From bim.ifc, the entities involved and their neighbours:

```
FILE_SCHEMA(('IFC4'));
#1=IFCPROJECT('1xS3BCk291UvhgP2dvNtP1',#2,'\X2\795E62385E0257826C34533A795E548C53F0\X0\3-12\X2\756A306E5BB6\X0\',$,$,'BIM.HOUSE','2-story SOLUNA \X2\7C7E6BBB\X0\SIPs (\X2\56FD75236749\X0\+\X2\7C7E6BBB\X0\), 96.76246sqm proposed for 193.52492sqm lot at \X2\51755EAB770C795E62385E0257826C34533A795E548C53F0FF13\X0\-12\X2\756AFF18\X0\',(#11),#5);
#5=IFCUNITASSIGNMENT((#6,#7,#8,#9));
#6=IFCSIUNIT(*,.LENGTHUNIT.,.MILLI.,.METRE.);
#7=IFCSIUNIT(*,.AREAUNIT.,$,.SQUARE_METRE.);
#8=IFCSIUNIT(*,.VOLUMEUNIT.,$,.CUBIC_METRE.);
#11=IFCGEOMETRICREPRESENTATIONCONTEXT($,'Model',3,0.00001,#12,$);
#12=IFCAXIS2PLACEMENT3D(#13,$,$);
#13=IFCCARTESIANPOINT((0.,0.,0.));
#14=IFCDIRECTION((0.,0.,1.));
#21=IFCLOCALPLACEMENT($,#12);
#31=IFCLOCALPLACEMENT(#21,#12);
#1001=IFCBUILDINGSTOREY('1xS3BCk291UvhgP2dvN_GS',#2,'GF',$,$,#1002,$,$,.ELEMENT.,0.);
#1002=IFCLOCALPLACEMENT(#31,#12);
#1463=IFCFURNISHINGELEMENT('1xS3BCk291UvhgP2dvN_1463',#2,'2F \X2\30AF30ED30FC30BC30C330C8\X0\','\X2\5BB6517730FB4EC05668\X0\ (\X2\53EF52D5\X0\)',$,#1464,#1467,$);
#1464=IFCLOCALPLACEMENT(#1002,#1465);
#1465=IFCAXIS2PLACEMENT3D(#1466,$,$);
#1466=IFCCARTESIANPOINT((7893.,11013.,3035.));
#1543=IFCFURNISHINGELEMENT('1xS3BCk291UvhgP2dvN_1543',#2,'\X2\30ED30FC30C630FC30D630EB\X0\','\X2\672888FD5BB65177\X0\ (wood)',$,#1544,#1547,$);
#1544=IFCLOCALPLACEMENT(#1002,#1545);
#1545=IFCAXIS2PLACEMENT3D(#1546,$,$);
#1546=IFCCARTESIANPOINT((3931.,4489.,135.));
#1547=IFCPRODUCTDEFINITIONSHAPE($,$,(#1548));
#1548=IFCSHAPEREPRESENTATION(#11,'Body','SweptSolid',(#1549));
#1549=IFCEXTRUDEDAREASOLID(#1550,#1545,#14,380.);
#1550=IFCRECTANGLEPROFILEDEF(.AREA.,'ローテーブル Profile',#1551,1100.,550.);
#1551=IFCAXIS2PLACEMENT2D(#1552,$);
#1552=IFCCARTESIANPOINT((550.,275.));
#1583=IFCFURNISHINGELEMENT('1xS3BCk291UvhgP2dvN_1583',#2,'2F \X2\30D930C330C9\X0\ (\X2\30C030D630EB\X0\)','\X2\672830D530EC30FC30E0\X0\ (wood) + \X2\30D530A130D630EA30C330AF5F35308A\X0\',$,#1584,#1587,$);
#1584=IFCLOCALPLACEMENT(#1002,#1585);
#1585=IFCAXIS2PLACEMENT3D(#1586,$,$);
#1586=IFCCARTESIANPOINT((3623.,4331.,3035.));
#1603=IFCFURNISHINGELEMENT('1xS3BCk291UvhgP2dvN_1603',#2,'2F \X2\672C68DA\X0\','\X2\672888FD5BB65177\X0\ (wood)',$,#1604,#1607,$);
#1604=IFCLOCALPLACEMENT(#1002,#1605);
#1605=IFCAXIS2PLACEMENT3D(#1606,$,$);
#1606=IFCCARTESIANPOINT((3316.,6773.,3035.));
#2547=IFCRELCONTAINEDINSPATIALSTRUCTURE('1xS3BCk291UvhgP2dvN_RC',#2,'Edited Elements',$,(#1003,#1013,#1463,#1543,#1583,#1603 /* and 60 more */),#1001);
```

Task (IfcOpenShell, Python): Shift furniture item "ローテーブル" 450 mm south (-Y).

```python
import ifcopenshell
import ifcopenshell.api.geometry
import ifcopenshell.util.placement
import ifcopenshell.util.unit

model = ifcopenshell.open("bim.ifc")
unit_scale = ifcopenshell.util.unit.calculate_unit_scale(model)

item = model.by_guid("1xS3BCk291UvhgP2dvN_1543")
matrix = ifcopenshell.util.placement.get_local_placement(item.ObjectPlacement)
matrix[1, 3] -= 0.45 / unit_scale
ifcopenshell.api.geometry.edit_object_placement(model, product=item, matrix=matrix, is_si=False)

print(ifcopenshell.util.placement.get_local_placement(item.ObjectPlacement).round(3) + 0.0)

model.write("bim_updated.ifc")
```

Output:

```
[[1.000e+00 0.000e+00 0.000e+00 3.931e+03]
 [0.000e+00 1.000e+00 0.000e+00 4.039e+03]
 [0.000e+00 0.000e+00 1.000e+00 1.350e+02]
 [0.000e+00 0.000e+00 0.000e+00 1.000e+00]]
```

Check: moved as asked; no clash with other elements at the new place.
